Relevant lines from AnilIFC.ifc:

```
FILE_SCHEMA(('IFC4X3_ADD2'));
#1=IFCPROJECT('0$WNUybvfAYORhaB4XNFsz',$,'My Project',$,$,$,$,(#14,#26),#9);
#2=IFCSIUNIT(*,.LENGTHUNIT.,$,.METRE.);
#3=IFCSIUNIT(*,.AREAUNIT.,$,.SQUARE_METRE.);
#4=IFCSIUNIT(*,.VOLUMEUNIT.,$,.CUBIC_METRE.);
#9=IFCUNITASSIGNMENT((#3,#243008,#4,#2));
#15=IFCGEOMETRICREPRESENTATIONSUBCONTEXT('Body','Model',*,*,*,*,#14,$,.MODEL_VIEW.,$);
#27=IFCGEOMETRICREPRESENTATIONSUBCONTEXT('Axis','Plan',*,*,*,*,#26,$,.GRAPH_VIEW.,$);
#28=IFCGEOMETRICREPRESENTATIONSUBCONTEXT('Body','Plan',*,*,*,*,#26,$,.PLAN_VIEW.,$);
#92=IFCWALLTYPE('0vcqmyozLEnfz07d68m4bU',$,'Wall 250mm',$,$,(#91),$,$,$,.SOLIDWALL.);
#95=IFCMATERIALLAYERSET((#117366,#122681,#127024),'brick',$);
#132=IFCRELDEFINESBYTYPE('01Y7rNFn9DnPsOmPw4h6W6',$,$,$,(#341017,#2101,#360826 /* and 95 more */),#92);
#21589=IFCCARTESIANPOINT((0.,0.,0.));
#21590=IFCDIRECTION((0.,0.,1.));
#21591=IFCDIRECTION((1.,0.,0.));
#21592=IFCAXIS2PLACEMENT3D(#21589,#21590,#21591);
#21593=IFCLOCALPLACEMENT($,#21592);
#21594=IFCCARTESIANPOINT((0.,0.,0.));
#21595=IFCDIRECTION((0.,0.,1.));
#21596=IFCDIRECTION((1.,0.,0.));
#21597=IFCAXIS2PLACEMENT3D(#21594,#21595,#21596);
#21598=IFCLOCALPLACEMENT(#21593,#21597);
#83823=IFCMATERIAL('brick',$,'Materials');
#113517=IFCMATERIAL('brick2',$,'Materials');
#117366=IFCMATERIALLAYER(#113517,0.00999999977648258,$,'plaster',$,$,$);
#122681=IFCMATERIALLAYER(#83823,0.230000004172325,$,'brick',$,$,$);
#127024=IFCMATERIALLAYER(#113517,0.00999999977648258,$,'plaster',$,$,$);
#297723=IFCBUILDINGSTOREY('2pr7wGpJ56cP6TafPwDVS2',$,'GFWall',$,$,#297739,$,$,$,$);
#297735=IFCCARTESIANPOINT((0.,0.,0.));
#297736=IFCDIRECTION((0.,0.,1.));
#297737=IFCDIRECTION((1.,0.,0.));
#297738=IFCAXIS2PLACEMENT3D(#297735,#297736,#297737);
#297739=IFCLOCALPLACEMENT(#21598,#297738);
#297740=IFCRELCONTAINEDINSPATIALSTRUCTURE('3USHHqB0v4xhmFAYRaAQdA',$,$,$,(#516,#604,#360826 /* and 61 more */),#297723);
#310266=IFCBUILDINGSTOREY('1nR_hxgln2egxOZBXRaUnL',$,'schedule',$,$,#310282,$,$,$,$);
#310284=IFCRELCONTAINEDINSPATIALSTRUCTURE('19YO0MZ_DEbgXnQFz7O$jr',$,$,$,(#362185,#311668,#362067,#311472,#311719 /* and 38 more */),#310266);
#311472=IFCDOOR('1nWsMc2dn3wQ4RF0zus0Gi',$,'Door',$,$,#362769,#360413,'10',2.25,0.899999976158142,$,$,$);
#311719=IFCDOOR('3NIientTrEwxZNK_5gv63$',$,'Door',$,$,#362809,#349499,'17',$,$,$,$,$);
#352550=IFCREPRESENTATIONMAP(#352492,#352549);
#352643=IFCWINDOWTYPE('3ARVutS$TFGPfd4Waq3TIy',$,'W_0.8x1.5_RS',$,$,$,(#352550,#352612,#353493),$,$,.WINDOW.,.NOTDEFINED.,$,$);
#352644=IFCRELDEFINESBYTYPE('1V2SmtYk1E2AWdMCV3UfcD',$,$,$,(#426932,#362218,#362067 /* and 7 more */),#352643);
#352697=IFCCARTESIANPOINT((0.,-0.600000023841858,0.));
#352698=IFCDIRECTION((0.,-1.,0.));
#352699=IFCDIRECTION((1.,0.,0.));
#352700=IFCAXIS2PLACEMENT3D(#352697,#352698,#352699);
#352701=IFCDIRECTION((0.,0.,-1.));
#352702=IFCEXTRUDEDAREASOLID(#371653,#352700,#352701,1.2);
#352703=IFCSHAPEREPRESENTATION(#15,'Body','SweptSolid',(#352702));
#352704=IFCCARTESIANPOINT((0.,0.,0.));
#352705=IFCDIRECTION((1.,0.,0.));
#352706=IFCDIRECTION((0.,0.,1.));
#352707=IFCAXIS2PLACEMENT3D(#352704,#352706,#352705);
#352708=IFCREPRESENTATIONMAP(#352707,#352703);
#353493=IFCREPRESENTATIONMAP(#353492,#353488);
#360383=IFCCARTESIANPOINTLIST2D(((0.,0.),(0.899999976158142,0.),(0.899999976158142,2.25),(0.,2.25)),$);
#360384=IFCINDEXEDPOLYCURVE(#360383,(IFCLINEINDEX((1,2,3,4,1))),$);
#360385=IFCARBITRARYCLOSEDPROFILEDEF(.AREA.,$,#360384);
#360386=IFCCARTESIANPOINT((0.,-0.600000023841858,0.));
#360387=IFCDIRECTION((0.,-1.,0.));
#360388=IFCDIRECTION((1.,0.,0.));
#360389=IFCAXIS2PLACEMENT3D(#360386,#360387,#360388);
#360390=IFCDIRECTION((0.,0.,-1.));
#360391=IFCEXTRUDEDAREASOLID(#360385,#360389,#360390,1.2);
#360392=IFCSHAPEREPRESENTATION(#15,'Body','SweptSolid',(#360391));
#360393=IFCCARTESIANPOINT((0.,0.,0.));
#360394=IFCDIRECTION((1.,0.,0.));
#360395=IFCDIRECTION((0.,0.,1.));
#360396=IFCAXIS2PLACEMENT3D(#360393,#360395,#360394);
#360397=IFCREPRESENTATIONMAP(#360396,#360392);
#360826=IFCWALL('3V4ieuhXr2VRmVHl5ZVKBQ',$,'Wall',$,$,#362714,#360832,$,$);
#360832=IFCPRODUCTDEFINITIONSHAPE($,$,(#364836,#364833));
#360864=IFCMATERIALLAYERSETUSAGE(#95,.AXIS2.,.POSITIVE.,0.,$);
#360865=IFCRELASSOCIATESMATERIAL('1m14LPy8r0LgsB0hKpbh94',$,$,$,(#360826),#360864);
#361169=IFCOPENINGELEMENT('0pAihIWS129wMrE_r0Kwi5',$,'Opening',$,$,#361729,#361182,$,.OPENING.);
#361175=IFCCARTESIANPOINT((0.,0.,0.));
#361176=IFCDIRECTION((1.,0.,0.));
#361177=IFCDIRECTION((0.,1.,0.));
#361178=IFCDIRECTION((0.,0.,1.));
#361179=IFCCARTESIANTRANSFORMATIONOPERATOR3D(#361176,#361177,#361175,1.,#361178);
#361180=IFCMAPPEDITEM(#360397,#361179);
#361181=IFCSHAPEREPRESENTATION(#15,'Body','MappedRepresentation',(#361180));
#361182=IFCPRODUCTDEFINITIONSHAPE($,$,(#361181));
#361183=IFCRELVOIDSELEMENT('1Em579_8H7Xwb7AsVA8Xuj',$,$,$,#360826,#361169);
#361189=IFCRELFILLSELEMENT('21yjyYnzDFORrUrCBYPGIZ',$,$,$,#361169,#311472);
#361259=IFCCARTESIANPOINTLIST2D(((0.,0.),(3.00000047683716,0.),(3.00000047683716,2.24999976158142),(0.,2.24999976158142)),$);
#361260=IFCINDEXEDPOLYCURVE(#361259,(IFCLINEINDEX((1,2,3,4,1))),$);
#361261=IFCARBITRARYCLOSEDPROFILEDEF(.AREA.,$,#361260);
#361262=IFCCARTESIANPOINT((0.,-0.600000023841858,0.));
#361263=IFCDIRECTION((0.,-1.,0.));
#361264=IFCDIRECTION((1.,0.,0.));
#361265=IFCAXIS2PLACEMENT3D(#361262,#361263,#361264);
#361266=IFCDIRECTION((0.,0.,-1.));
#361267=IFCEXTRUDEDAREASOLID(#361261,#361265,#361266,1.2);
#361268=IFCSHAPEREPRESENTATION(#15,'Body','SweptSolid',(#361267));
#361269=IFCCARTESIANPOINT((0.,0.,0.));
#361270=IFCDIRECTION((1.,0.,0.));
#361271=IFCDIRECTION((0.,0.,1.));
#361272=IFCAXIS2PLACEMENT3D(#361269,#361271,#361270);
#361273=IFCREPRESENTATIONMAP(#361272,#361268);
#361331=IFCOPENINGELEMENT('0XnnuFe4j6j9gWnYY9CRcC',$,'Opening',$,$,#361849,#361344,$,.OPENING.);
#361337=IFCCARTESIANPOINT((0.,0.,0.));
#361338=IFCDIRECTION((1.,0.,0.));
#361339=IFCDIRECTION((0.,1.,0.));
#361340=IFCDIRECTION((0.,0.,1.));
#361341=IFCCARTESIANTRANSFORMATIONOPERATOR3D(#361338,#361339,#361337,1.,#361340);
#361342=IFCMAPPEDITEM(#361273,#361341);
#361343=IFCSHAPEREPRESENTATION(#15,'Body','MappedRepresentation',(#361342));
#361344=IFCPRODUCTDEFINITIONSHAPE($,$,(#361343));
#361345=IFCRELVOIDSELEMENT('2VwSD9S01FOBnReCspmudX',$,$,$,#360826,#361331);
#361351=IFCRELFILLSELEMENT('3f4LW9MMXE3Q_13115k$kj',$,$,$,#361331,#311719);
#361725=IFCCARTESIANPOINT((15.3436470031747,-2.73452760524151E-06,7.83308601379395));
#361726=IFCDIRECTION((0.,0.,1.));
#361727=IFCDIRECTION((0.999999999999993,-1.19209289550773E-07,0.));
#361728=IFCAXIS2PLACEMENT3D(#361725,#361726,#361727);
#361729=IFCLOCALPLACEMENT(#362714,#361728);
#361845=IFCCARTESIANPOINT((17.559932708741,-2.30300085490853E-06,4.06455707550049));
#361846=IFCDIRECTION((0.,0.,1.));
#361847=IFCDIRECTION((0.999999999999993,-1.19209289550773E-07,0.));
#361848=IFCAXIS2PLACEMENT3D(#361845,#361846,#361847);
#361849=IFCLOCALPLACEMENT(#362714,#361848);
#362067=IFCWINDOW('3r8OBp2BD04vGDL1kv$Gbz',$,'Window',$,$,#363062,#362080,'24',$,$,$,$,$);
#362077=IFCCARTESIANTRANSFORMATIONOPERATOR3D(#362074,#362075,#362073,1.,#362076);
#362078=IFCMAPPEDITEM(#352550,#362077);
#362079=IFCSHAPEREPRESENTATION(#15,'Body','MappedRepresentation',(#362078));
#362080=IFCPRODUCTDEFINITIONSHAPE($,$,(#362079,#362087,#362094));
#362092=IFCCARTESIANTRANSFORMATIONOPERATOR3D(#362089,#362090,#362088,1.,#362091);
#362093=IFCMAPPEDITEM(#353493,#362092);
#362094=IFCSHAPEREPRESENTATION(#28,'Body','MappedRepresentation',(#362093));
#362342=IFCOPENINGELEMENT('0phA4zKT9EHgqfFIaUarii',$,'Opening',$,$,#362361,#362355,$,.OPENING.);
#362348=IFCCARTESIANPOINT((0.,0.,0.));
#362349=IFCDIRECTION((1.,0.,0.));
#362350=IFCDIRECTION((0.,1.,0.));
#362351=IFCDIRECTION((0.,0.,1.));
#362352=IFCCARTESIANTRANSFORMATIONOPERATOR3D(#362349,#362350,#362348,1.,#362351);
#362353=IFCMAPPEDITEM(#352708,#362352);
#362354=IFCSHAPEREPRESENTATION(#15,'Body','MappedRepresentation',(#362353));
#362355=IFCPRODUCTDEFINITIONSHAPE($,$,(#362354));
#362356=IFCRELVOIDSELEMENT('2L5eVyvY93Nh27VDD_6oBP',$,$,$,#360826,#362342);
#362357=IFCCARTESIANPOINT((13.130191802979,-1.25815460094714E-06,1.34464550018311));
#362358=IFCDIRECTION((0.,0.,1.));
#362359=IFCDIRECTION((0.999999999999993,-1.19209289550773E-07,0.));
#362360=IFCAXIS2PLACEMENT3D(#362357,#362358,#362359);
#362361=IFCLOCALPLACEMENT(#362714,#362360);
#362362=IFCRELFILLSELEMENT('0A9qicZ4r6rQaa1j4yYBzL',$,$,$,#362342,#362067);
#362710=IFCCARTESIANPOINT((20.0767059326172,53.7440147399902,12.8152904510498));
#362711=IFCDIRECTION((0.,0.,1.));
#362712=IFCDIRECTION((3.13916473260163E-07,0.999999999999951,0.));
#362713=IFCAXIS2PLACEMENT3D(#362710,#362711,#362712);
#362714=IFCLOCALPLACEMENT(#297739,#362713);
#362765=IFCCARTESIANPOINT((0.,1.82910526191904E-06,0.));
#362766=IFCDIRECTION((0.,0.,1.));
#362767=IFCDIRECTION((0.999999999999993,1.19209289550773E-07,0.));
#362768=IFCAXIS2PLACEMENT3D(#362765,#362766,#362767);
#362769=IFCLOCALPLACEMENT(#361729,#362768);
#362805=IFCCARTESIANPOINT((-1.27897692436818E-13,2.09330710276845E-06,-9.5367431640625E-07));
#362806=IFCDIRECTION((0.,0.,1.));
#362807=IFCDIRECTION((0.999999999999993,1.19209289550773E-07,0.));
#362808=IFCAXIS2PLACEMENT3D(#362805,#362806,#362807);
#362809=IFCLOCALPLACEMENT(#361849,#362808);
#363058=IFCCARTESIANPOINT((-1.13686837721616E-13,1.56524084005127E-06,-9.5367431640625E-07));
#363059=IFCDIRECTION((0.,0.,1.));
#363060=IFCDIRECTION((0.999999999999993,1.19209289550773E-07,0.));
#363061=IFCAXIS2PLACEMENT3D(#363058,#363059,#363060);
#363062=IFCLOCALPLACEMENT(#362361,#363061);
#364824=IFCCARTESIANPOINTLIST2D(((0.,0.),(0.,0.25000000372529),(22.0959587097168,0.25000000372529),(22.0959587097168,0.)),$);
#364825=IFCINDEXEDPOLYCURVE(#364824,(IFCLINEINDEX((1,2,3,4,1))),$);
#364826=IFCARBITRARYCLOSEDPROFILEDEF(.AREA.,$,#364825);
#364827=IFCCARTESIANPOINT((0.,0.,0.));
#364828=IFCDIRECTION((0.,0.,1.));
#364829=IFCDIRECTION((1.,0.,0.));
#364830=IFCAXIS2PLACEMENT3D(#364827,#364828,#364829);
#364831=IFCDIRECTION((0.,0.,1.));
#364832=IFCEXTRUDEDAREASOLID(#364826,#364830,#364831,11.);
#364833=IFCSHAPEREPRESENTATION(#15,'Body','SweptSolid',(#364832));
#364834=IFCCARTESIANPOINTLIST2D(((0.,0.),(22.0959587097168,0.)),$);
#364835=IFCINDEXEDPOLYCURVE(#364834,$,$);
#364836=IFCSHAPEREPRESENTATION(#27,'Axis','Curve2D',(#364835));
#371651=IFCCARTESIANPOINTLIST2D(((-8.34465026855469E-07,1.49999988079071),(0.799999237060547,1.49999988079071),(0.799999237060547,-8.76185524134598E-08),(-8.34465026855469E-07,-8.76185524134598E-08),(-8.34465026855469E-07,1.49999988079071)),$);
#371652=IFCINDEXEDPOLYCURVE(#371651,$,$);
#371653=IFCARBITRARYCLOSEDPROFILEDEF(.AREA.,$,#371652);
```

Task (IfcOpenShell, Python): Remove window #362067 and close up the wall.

```python
import ifcopenshell
import ifcopenshell.api.feature
import ifcopenshell.api.root
import ifcopenshell.geom
import ifcopenshell.util.shape

model = ifcopenshell.open("AnilIFC.ifc")
settings = ifcopenshell.geom.settings()


def volume(element):
    """Net volume in cubic metres, openings subtracted."""
    shape = ifcopenshell.geom.create_shape(settings, element)
    return ifcopenshell.util.shape.get_volume(shape.geometry)


window = model.by_id(362067)
opening = window.FillsVoids[0].RelatingOpeningElement
wall = opening.VoidsElements[0].RelatingBuildingElement
before = volume(wall)

ifcopenshell.api.root.remove_product(model, product=window)
ifcopenshell.api.feature.remove_feature(model, feature=opening)

after = volume(wall)

print(f"wall volume {before:.3f} -> {after:.3f} m3")

model.write("AnilIFC_updated.ifc")
```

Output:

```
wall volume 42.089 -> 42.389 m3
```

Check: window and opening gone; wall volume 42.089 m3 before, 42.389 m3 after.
